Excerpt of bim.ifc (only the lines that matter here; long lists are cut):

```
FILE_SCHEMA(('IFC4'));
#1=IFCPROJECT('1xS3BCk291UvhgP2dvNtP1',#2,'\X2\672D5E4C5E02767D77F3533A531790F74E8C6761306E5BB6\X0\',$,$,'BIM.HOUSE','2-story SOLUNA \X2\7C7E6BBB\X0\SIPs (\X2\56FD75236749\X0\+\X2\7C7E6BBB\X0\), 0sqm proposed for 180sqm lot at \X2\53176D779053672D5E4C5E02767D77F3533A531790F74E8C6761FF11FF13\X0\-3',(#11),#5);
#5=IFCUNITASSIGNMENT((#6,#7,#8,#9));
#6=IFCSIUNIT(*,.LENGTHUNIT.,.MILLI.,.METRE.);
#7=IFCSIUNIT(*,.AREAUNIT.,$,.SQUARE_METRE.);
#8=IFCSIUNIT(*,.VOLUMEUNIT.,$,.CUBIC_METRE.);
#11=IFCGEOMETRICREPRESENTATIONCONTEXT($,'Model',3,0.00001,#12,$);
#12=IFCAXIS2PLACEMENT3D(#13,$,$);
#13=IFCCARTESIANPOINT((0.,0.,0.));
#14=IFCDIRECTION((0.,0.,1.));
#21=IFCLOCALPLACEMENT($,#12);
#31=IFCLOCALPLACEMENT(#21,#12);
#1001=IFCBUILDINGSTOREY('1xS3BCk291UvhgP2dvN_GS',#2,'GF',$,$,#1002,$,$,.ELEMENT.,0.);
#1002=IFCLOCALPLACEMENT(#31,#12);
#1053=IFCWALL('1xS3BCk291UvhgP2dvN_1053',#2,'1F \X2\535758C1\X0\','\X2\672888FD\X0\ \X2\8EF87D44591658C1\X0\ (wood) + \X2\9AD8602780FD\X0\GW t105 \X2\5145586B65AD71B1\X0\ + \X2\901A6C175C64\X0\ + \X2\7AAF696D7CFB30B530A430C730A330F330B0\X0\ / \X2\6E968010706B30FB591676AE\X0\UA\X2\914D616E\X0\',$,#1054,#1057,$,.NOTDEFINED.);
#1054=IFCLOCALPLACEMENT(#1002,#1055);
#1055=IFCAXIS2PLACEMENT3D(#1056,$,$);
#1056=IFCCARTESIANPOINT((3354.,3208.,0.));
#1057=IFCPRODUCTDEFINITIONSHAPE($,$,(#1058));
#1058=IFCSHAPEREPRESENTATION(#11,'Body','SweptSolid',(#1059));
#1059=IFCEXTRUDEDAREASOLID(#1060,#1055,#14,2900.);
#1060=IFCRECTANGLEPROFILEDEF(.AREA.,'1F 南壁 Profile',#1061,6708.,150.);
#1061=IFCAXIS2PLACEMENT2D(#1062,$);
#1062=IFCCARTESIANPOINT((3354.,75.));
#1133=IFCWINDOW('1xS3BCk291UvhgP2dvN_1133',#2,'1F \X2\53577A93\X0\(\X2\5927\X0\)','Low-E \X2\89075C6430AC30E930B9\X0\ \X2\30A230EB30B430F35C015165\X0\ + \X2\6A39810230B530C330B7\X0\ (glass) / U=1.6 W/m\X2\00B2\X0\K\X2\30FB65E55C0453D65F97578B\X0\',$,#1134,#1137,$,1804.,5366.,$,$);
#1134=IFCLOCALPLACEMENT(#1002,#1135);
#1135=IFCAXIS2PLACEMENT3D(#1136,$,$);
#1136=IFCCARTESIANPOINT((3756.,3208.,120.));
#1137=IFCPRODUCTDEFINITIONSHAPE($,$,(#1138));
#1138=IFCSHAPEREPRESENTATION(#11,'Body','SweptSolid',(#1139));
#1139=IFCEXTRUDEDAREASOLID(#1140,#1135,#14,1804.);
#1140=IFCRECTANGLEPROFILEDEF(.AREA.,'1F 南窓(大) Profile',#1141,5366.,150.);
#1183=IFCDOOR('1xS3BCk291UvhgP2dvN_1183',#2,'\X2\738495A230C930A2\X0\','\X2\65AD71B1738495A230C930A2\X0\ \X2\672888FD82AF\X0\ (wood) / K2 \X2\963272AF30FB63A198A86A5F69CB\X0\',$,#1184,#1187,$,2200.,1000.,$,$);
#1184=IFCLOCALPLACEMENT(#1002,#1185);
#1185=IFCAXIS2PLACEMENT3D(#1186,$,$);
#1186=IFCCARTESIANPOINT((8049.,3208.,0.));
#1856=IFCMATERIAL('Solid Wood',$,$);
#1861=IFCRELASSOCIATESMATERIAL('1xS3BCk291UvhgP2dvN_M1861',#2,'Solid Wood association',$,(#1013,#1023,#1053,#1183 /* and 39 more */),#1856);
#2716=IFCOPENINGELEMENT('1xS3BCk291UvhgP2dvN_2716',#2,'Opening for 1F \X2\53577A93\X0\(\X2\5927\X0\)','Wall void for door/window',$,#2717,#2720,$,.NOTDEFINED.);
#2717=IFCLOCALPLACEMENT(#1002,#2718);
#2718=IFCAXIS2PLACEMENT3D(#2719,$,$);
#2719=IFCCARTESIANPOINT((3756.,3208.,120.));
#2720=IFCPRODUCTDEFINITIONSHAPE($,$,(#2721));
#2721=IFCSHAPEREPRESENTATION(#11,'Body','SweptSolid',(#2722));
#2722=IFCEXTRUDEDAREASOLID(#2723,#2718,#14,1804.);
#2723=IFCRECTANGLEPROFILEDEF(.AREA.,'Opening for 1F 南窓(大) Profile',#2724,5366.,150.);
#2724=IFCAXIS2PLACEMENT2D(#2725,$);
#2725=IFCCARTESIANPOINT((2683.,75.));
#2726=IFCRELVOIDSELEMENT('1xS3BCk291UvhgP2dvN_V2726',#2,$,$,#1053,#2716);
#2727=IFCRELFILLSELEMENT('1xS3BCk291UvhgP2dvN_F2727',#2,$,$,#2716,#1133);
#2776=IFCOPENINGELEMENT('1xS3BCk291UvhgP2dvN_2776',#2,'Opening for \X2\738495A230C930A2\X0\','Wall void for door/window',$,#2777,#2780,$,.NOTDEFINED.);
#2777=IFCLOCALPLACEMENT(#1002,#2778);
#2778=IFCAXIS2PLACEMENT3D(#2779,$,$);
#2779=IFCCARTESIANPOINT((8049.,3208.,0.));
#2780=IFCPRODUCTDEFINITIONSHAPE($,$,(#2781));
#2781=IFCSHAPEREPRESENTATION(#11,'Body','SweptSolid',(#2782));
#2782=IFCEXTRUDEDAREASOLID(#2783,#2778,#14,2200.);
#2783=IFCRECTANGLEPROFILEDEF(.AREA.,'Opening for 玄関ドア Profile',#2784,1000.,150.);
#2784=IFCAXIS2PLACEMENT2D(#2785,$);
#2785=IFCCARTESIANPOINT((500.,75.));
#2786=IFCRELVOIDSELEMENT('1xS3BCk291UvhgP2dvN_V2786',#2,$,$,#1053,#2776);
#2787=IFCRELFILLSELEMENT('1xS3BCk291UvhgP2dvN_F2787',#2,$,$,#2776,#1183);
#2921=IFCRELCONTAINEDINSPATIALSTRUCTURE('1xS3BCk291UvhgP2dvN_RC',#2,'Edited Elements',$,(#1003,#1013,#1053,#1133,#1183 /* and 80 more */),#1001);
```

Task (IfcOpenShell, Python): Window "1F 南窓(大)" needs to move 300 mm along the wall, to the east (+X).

```python
import ifcopenshell
import ifcopenshell.api.geometry
import ifcopenshell.util.placement
import ifcopenshell.util.unit

model = ifcopenshell.open("bim.ifc")
unit_scale = ifcopenshell.util.unit.calculate_unit_scale(model)

window = model.by_guid("1xS3BCk291UvhgP2dvN_1133")
opening = window.FillsVoids[0].RelatingOpeningElement
wall = opening.VoidsElements[0].RelatingBuildingElement

wall_matrix = ifcopenshell.util.placement.get_local_placement(wall.ObjectPlacement)
shift = wall_matrix[:3, 0] * 0.3 / unit_scale
before = ifcopenshell.util.placement.get_local_placement(window.ObjectPlacement)[:3, 3].copy()

# The window is not placed relative to its opening, so move both.
for product in (opening, window):
    matrix = ifcopenshell.util.placement.get_local_placement(product.ObjectPlacement)
    matrix[:3, 3] += shift
    ifcopenshell.api.geometry.edit_object_placement(model, product=product, matrix=matrix, is_si=False)

after = ifcopenshell.util.placement.get_local_placement(window.ObjectPlacement)[:3, 3]
print("window moved by", (after - before).round(3) + 0.0)

model.write("bim_edited.ifc")
```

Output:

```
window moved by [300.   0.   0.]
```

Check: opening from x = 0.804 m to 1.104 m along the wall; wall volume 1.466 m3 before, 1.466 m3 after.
